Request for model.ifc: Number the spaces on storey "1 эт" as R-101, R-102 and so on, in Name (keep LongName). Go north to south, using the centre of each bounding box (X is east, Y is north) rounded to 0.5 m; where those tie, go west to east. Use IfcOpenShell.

First a look at what the model holds.

```python
import ifcopenshell
import ifcopenshell.util.element
import ifcopenshell.util.placement

model = ifcopenshell.open("model.ifc")
print(model.schema)
storey = next(s for s in model.by_type("IfcBuildingStorey") if s.Name == "1 эт")
spaces = [e for e in ifcopenshell.util.element.get_decomposition(storey) if e.is_a("IfcSpace")]
for e in sorted(spaces, key=lambda e: e.id()):
    origin = ifcopenshell.util.placement.get_local_placement(e.ObjectPlacement)[:3, 3]
    print(e.id(), e.Name, e.LongName, origin.round(2) + 0.0, sep=" | ")
```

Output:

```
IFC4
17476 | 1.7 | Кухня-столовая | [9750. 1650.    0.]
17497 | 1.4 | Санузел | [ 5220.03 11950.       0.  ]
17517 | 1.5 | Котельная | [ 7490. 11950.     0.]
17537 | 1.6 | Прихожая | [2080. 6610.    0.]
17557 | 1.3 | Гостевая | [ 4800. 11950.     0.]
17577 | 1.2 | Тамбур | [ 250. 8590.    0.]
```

```python
import ifcopenshell
import ifcopenshell.geom
import ifcopenshell.util.element
import ifcopenshell.util.shape

model = ifcopenshell.open("model.ifc")
settings = ifcopenshell.geom.settings()
settings.set("use-world-coords", True)


def centre(element):
    shape = ifcopenshell.geom.create_shape(settings, element)
    return ifcopenshell.util.shape.get_bbox_centroid(shape.geometry)


storey = next(s for s in model.by_type("IfcBuildingStorey") if s.Name == "1 эт")
spaces = [e for e in ifcopenshell.util.element.get_decomposition(storey) if e.is_a("IfcSpace")]

# Insertion points can sit at a corner or the storey origin, so sort by the geometry (in metres).
centres = {e: centre(e) for e in spaces}
spaces.sort(key=lambda e: (-round(centres[e][1] / 0.5), centres[e][0]))

for i, e in enumerate(spaces, start=1):
    number = f"R-1{i:02d}"
    e.Name = number
    print(e.id(), number)

model.write("model_updated.ifc")
```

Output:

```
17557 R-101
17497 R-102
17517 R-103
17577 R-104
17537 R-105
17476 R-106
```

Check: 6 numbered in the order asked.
